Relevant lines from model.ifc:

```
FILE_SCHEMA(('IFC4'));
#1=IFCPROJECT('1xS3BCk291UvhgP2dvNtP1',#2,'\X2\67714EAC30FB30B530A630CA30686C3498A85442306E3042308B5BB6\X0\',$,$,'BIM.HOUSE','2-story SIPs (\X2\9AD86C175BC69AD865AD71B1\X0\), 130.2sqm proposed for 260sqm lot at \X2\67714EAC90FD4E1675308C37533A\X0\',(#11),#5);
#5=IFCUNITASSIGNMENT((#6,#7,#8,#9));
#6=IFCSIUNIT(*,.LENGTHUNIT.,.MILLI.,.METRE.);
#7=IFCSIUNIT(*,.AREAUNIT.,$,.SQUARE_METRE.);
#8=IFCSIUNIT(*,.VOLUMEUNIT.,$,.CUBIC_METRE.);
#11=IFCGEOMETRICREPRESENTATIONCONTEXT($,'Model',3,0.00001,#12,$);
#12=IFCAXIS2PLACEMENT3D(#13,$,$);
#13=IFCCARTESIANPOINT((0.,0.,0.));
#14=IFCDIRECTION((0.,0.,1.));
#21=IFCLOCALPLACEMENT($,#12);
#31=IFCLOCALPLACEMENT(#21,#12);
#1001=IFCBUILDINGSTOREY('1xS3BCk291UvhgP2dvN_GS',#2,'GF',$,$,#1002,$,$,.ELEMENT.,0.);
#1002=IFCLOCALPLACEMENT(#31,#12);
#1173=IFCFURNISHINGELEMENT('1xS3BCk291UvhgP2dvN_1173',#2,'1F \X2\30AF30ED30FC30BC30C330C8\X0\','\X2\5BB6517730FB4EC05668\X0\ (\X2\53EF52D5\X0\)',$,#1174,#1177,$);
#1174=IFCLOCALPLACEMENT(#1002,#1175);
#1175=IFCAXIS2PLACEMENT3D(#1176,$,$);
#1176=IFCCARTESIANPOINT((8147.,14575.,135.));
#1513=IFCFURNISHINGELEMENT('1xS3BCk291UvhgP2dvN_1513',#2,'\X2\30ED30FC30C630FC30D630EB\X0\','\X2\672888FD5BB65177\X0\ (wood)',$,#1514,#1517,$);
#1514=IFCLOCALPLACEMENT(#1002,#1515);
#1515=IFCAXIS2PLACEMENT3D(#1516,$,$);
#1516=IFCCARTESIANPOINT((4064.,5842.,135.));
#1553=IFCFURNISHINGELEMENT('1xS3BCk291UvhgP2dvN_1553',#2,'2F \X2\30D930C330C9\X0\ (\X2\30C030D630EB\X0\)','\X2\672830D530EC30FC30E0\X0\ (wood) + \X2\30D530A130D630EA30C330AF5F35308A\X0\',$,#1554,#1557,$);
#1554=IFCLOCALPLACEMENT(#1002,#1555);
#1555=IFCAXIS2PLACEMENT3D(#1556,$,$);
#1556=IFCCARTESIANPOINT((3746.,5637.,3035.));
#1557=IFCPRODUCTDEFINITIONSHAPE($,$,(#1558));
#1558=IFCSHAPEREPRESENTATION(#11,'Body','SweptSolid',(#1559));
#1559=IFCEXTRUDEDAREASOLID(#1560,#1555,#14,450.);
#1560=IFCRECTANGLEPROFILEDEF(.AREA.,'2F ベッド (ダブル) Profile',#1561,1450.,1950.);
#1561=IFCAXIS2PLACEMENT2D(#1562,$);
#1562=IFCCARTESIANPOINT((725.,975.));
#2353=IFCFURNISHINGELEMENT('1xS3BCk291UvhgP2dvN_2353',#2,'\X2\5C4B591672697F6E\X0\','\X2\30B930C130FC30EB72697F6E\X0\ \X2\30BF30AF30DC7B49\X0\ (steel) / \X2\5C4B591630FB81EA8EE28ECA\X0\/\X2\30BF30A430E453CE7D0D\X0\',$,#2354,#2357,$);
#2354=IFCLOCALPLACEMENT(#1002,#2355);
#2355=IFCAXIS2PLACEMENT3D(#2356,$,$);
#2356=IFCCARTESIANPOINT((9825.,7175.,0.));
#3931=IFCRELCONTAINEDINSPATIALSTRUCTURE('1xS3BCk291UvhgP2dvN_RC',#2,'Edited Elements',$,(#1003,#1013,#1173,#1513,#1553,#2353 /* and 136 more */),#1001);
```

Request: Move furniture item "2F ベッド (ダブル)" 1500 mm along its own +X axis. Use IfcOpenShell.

```python
import ifcopenshell
import ifcopenshell.api.geometry
import ifcopenshell.util.placement

model = ifcopenshell.open("model.ifc")

item = model.by_guid("1xS3BCk291UvhgP2dvN_1553")
matrix = ifcopenshell.util.placement.get_local_placement(item.ObjectPlacement)
matrix[:3, 3] += matrix[:3, 0] * 1500.0
ifcopenshell.api.geometry.edit_object_placement(model, product=item, matrix=matrix, is_si=False)

print(ifcopenshell.util.placement.get_local_placement(item.ObjectPlacement).round(3) + 0.0)

model.write("model_updated.ifc")
```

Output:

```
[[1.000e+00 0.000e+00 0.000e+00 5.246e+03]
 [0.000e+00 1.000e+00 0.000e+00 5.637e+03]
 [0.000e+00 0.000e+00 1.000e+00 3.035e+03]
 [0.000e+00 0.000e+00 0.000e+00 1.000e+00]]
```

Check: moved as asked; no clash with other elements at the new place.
